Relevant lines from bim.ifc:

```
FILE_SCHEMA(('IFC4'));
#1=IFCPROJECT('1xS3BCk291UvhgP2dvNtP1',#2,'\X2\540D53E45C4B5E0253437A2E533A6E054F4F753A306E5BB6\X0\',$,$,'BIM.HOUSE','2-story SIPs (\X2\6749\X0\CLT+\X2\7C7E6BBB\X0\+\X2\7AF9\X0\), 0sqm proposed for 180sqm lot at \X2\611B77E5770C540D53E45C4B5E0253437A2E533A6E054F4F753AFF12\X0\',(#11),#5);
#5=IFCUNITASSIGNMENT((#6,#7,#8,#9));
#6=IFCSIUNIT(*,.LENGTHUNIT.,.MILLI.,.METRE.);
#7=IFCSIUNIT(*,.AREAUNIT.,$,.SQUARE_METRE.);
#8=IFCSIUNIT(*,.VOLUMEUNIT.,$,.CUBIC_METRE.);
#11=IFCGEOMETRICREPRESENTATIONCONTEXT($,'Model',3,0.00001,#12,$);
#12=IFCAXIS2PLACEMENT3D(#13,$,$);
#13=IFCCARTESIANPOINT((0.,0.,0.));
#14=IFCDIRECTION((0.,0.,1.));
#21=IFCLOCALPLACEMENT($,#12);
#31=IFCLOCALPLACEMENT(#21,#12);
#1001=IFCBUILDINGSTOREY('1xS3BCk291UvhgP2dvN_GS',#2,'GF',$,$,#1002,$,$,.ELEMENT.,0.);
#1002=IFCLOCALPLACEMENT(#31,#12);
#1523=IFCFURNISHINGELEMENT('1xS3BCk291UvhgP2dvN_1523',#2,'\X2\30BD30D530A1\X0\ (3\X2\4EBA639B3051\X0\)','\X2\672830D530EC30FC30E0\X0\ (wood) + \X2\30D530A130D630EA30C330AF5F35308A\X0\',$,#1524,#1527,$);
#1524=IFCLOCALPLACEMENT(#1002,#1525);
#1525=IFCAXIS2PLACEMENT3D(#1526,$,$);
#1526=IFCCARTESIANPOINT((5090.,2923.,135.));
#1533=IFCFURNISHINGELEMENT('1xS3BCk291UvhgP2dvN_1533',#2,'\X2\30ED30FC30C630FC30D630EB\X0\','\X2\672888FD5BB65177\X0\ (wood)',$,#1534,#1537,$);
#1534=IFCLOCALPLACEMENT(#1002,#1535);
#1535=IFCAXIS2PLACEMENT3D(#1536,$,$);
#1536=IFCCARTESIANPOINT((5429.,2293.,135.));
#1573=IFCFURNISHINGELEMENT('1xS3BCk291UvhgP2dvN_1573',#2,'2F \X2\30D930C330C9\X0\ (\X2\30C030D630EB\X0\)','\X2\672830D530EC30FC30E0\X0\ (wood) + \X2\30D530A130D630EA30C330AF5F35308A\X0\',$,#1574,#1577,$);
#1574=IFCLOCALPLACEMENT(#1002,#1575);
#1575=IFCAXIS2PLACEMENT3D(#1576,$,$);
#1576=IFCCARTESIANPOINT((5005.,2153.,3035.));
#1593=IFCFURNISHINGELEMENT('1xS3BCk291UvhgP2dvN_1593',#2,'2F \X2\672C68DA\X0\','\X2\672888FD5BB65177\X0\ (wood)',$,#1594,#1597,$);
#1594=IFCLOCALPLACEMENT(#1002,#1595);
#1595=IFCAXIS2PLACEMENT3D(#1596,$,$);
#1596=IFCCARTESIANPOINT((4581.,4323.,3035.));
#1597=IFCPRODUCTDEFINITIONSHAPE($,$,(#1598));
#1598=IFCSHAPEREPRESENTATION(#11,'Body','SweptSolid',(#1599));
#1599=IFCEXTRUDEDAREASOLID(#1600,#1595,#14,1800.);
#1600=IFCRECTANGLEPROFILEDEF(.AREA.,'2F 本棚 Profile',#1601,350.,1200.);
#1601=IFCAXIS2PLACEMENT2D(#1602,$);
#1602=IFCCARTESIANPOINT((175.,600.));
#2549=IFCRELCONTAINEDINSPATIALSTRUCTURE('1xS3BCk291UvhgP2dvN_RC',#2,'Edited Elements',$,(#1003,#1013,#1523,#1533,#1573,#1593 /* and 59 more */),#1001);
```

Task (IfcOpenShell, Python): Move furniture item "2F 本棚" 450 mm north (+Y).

```python
import ifcopenshell
import ifcopenshell.api.geometry
import ifcopenshell.util.placement
import ifcopenshell.util.unit

model = ifcopenshell.open("bim.ifc")
unit_scale = ifcopenshell.util.unit.calculate_unit_scale(model)

item = model.by_guid("1xS3BCk291UvhgP2dvN_1593")
matrix = ifcopenshell.util.placement.get_local_placement(item.ObjectPlacement)
matrix[1, 3] += 0.45 / unit_scale
ifcopenshell.api.geometry.edit_object_placement(model, product=item, matrix=matrix, is_si=False)

print(ifcopenshell.util.placement.get_local_placement(item.ObjectPlacement).round(3) + 0.0)

model.write("bim-out.ifc")
```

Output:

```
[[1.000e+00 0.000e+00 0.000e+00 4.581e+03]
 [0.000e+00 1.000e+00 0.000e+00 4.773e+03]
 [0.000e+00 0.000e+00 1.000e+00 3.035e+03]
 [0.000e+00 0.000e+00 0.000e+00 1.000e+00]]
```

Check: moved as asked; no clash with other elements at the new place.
